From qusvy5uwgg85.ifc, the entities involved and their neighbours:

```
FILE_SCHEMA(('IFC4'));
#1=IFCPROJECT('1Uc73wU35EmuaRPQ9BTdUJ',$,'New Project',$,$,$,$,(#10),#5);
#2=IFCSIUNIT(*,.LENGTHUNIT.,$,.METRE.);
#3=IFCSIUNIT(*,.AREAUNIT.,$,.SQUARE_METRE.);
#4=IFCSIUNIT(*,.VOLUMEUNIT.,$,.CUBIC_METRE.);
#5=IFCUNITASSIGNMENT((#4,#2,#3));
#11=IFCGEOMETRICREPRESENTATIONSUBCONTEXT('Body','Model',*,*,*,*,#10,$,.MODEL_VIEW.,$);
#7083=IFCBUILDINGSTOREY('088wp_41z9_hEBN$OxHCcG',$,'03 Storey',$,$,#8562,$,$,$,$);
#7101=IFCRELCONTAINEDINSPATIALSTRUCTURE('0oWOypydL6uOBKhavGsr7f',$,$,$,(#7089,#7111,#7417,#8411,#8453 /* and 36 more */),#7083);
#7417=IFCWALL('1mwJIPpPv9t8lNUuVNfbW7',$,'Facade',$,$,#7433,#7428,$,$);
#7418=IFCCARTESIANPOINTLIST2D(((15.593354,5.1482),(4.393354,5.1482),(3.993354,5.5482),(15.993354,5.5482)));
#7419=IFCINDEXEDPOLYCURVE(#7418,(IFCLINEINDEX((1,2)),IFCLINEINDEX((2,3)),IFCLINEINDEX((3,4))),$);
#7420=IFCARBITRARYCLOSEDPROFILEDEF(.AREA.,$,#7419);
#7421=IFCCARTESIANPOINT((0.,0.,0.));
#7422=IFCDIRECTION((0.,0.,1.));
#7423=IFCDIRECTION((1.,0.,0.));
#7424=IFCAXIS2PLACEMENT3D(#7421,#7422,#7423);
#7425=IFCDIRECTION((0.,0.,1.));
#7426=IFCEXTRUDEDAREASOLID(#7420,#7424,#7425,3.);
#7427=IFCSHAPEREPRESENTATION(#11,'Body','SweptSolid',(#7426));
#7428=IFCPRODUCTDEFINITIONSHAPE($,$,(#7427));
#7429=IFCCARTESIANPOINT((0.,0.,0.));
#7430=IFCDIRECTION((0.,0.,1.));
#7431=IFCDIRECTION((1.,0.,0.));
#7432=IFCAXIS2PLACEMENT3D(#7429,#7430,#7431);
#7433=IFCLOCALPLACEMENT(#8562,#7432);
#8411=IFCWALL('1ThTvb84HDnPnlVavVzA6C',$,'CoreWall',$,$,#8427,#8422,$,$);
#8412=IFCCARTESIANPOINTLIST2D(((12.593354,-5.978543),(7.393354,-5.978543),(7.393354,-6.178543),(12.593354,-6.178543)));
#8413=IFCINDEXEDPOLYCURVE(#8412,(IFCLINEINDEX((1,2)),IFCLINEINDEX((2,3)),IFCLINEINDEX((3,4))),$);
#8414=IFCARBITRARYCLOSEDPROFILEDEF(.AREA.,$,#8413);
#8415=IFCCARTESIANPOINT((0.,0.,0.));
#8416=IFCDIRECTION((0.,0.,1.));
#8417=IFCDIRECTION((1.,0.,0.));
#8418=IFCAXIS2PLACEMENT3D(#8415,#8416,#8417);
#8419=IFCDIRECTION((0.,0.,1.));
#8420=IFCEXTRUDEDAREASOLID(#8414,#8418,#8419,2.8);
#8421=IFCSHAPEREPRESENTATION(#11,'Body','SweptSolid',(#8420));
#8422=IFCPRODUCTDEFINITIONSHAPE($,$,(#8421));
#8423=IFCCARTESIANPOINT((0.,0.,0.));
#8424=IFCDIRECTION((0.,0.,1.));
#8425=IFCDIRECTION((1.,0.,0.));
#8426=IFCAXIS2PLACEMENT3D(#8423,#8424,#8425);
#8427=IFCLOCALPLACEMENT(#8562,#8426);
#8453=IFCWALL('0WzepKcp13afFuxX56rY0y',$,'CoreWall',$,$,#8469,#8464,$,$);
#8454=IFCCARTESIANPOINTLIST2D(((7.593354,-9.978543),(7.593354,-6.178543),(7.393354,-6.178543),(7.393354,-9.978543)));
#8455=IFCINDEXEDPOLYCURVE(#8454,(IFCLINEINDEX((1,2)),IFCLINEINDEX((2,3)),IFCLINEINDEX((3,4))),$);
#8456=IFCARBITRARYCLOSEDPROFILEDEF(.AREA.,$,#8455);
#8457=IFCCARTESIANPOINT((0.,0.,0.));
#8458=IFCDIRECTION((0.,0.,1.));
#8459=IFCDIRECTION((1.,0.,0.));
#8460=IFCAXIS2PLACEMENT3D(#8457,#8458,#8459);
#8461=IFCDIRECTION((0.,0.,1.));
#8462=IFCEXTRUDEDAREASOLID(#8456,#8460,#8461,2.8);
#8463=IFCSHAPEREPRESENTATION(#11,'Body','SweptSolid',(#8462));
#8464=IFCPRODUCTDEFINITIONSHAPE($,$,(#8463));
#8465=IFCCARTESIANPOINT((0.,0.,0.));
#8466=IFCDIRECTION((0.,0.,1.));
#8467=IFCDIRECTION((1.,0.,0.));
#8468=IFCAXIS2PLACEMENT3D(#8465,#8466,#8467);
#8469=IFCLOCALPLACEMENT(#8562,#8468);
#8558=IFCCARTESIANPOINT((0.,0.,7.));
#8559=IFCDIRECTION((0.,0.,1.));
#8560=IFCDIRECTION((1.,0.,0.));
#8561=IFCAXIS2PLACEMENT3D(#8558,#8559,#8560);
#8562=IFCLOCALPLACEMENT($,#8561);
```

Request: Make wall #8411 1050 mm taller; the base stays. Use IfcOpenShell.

```python
import ifcopenshell
import ifcopenshell.geom
import ifcopenshell.util.representation
import ifcopenshell.util.shape

model = ifcopenshell.open("qusvy5uwgg85.ifc")
settings = ifcopenshell.geom.settings()


def volume(element):
    """Net volume in cubic metres, openings subtracted."""
    shape = ifcopenshell.geom.create_shape(settings, element)
    return ifcopenshell.util.shape.get_volume(shape.geometry)


wall = model.by_guid("1ThTvb84HDnPnlVavVzA6C")
before = volume(wall)

body = ifcopenshell.util.representation.get_representation(wall, "Model", "Body")
solid = body.Items[0]
old_height = solid.Depth
solid.Depth += 1.05
after = volume(wall)

print(f"height {old_height:g} -> {solid.Depth:g}, volume {before:.3f} -> {after:.3f} m3")

model.write("qusvy5uwgg85_rev.ifc")
```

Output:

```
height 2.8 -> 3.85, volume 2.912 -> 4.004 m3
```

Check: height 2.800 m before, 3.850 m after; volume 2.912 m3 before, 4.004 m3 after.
